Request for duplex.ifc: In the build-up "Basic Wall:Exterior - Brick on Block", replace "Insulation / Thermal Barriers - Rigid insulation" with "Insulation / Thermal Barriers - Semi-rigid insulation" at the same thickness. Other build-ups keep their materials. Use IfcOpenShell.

First a look at what the model holds.

```python
import ifcopenshell
import ifcopenshell.util.element

model = ifcopenshell.open("duplex.ifc")
print(model.schema)
for layer_set in model.by_type("IfcMaterialLayerSet"):
    if layer_set.LayerSetName == "Basic Wall:Exterior - Brick on Block":
        for layer in layer_set.MaterialLayers:
            print(layer.id(), layer.Material and layer.Material.Name, layer.LayerThickness, sep=" | ")
        print(len(ifcopenshell.util.element.get_elements_by_material(model, layer_set)), "elements and types use it")
print(sorted(m.Name for m in model.by_type("IfcMaterial") if m.Name)[:60])
```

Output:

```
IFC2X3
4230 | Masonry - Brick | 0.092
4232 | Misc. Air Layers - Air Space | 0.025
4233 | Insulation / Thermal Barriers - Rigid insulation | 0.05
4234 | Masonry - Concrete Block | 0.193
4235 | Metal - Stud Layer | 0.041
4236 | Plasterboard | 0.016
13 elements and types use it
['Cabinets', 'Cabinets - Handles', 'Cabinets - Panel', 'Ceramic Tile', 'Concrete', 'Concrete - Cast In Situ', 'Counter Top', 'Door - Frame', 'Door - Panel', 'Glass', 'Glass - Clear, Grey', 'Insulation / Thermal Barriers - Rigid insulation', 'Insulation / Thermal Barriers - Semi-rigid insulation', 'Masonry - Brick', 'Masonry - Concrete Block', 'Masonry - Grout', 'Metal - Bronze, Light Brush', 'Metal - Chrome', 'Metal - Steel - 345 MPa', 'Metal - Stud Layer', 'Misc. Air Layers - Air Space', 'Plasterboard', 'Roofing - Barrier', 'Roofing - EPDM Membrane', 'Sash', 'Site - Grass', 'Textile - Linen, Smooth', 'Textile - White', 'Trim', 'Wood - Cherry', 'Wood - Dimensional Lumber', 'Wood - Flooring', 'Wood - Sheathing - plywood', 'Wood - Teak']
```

```python
import ifcopenshell
import ifcopenshell.api.material

model = ifcopenshell.open("duplex.ifc")

layer_set = next(s for s in model.by_type("IfcMaterialLayerSet") if s.LayerSetName == "Basic Wall:Exterior - Brick on Block")
layer = next(l for l in layer_set.MaterialLayers if l.Material and l.Material.Name == "Insulation / Thermal Barriers - Rigid insulation")
material = next(m for m in model.by_type("IfcMaterial") if m.Name == "Insulation / Thermal Barriers - Semi-rigid insulation")

# Point this one layer at the other material; renaming the old one would change it everywhere.
ifcopenshell.api.material.edit_layer(model, layer=layer, attributes={}, material=material)

print([l.Material.Name if l.Material else None for l in layer_set.MaterialLayers])

model.write("duplex_edited.ifc")
```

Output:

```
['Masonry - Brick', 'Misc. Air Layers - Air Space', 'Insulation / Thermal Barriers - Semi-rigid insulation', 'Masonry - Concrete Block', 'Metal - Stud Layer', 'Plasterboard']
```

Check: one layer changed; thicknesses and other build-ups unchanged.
